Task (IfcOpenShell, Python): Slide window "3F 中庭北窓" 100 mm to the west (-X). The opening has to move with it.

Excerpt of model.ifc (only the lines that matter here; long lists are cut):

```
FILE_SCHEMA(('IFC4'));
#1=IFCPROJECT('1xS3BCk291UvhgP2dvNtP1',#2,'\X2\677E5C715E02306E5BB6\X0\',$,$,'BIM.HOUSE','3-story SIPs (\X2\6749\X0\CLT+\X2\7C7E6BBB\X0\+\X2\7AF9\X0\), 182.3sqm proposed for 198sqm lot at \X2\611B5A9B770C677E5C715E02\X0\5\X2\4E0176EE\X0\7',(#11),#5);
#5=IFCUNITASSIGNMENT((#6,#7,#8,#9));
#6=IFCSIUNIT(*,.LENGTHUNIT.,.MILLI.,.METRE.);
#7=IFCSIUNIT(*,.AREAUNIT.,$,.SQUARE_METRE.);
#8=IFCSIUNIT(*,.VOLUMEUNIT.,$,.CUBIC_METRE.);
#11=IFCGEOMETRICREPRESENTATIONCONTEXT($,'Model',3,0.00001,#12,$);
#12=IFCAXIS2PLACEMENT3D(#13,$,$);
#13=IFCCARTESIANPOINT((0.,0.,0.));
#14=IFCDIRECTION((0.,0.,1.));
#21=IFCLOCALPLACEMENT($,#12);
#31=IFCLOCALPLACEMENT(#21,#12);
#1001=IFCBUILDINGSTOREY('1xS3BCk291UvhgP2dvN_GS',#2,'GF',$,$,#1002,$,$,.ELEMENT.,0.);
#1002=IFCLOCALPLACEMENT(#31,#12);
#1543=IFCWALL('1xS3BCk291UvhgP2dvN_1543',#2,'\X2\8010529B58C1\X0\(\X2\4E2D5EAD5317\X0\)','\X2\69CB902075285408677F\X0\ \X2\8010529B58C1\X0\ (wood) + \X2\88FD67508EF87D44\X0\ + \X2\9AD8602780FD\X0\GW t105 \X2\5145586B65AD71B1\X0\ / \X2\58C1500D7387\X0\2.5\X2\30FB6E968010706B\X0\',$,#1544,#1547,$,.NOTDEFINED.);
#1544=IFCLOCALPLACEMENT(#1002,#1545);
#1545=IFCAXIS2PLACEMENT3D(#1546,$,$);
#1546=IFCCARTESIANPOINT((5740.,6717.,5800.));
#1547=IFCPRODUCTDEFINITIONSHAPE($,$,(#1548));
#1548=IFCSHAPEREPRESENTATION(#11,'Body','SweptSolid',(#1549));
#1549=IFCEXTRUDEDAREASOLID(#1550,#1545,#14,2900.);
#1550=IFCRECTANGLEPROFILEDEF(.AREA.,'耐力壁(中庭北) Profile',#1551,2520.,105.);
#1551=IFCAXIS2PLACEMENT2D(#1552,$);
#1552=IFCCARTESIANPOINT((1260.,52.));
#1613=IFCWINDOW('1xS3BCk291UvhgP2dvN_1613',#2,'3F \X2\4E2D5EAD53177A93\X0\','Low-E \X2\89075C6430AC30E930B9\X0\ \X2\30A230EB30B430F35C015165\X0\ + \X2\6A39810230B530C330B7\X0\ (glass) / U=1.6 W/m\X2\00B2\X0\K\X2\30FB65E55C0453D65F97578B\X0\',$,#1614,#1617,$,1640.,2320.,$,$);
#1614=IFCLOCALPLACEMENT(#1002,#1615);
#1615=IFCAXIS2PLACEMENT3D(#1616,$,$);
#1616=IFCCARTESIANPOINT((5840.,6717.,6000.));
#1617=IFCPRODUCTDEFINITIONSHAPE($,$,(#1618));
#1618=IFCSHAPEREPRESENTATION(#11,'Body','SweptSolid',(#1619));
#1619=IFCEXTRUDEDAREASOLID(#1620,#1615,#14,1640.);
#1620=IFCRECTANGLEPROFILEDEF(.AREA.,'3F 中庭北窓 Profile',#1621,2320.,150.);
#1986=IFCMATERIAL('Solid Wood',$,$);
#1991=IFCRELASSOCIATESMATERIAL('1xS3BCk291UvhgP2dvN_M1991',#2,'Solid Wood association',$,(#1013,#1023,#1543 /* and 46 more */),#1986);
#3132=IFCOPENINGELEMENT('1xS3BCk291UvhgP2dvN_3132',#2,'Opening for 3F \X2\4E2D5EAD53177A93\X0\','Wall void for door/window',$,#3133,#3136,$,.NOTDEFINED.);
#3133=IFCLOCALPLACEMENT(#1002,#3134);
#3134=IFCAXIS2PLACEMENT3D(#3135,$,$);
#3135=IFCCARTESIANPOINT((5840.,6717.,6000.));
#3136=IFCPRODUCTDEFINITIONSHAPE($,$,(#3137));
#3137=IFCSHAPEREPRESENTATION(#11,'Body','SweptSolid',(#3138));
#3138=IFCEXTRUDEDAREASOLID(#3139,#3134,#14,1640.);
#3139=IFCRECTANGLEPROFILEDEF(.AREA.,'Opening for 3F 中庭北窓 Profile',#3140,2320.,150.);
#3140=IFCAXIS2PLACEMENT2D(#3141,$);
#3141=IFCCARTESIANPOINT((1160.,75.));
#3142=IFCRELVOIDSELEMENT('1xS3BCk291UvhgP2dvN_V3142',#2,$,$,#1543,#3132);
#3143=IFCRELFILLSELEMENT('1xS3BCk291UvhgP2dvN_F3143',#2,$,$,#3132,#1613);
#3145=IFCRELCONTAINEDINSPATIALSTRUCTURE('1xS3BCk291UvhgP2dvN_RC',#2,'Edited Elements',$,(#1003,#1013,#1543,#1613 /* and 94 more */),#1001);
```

```python
import ifcopenshell
import ifcopenshell.api.geometry
import ifcopenshell.util.placement
import ifcopenshell.util.unit

model = ifcopenshell.open("model.ifc")
unit_scale = ifcopenshell.util.unit.calculate_unit_scale(model)

window = model.by_id(1613)
opening = window.FillsVoids[0].RelatingOpeningElement
wall = opening.VoidsElements[0].RelatingBuildingElement

wall_matrix = ifcopenshell.util.placement.get_local_placement(wall.ObjectPlacement)
shift = wall_matrix[:3, 0] * -0.1 / unit_scale
before = ifcopenshell.util.placement.get_local_placement(window.ObjectPlacement)[:3, 3].copy()

# The window is not placed relative to its opening, so move both.
for product in (opening, window):
    matrix = ifcopenshell.util.placement.get_local_placement(product.ObjectPlacement)
    matrix[:3, 3] += shift
    ifcopenshell.api.geometry.edit_object_placement(model, product=product, matrix=matrix, is_si=False)

after = ifcopenshell.util.placement.get_local_placement(window.ObjectPlacement)[:3, 3]
print("window moved by", (after - before).round(3) + 0.0)

model.write("model_rev.ifc")
```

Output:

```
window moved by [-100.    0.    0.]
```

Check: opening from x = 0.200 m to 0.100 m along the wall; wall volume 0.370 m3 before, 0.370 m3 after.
